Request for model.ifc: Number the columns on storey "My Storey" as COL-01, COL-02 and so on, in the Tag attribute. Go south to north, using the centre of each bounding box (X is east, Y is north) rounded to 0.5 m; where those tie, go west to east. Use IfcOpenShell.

First a look at what the model holds.

```python
import ifcopenshell
import ifcopenshell.util.element
import ifcopenshell.util.placement

model = ifcopenshell.open("model.ifc")
print(model.schema)
storey = next(s for s in model.by_type("IfcBuildingStorey") if s.Name == "My Storey")
columns = [e for e in ifcopenshell.util.element.get_decomposition(storey) if e.is_a("IfcColumn")]
for e in sorted(columns, key=lambda e: e.id()):
    origin = ifcopenshell.util.placement.get_local_placement(e.ObjectPlacement)[:3, 3]
    print(e.id(), e.Tag, e.Name, origin.round(2) + 0.0, sep=" | ")
```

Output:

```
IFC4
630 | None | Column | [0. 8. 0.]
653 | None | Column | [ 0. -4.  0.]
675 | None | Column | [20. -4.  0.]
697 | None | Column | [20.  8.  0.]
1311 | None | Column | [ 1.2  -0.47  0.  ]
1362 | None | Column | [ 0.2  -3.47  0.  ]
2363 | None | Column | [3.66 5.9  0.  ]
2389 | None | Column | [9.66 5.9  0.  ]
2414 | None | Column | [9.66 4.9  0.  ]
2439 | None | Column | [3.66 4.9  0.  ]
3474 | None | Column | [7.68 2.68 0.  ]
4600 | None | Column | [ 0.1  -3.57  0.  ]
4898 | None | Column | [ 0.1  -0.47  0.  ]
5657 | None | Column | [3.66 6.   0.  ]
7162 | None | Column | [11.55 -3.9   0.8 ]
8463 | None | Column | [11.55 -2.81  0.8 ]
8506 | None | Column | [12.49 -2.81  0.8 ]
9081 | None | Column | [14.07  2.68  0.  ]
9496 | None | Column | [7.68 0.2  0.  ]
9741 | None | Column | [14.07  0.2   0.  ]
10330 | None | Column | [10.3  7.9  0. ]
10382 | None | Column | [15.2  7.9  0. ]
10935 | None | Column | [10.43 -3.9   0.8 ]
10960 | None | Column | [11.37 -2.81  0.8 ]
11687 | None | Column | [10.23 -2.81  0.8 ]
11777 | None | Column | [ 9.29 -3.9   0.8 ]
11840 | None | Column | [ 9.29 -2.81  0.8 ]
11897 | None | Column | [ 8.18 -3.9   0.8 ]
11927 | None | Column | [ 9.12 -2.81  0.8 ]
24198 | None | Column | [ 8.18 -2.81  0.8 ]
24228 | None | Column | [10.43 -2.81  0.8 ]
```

```python
import ifcopenshell
import ifcopenshell.geom
import ifcopenshell.util.element
import ifcopenshell.util.shape

model = ifcopenshell.open("model.ifc")
settings = ifcopenshell.geom.settings()
settings.set("use-world-coords", True)


def centre(element):
    shape = ifcopenshell.geom.create_shape(settings, element)
    return ifcopenshell.util.shape.get_bbox_centroid(shape.geometry)


storey = next(s for s in model.by_type("IfcBuildingStorey") if s.Name == "My Storey")
columns = [e for e in ifcopenshell.util.element.get_decomposition(storey) if e.is_a("IfcColumn")]

# Insertion points can sit at a corner or the storey origin, so sort by the geometry (in metres).
centres = {e: centre(e) for e in columns}
columns.sort(key=lambda e: (round(centres[e][1] / 0.5), centres[e][0]))

for i, e in enumerate(columns, start=1):
    number = f"COL-{i:02d}"
    e.Tag = number
    print(e.id(), number)

model.write("model_edited.ifc")
```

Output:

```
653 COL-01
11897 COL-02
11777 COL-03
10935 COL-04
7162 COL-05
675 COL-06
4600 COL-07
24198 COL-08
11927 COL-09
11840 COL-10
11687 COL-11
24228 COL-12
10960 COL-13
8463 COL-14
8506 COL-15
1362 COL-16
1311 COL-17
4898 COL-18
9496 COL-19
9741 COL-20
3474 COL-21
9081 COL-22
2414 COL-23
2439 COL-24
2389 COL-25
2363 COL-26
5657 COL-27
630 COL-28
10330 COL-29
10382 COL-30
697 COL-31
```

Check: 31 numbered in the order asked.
